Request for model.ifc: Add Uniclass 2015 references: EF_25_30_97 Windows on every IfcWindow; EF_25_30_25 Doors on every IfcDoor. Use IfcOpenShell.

First a look at what the model holds.

```python
import ifcopenshell

model = ifcopenshell.open("model.ifc")
print(model.schema)
print("classifications:", [c.Name for c in model.by_type("IfcClassification")])
for ifc_class in ("IfcDoor", "IfcRoof", "IfcStair", "IfcWall", "IfcWindow"):
    print(ifc_class, len(model.by_type(ifc_class)))
```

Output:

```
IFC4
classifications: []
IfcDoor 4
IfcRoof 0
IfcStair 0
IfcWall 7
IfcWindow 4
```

```python
import ifcopenshell
import ifcopenshell.api.classification

model = ifcopenshell.open("model.ifc")

system = ifcopenshell.api.classification.add_classification(model, classification="Uniclass 2015")

codes = {
    "IfcWindow": ("EF_25_30_97", "Windows"),
    "IfcDoor": ("EF_25_30_25", "Doors"),
}
for ifc_class, (code, name) in codes.items():
    products = model.by_type(ifc_class)
    ifcopenshell.api.classification.add_reference(
        model, products=products, classification=system, identification=code, name=name
    )
    print(code, len(products))

model.write("model_v2.ifc")
```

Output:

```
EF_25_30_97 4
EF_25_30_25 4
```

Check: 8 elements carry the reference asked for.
